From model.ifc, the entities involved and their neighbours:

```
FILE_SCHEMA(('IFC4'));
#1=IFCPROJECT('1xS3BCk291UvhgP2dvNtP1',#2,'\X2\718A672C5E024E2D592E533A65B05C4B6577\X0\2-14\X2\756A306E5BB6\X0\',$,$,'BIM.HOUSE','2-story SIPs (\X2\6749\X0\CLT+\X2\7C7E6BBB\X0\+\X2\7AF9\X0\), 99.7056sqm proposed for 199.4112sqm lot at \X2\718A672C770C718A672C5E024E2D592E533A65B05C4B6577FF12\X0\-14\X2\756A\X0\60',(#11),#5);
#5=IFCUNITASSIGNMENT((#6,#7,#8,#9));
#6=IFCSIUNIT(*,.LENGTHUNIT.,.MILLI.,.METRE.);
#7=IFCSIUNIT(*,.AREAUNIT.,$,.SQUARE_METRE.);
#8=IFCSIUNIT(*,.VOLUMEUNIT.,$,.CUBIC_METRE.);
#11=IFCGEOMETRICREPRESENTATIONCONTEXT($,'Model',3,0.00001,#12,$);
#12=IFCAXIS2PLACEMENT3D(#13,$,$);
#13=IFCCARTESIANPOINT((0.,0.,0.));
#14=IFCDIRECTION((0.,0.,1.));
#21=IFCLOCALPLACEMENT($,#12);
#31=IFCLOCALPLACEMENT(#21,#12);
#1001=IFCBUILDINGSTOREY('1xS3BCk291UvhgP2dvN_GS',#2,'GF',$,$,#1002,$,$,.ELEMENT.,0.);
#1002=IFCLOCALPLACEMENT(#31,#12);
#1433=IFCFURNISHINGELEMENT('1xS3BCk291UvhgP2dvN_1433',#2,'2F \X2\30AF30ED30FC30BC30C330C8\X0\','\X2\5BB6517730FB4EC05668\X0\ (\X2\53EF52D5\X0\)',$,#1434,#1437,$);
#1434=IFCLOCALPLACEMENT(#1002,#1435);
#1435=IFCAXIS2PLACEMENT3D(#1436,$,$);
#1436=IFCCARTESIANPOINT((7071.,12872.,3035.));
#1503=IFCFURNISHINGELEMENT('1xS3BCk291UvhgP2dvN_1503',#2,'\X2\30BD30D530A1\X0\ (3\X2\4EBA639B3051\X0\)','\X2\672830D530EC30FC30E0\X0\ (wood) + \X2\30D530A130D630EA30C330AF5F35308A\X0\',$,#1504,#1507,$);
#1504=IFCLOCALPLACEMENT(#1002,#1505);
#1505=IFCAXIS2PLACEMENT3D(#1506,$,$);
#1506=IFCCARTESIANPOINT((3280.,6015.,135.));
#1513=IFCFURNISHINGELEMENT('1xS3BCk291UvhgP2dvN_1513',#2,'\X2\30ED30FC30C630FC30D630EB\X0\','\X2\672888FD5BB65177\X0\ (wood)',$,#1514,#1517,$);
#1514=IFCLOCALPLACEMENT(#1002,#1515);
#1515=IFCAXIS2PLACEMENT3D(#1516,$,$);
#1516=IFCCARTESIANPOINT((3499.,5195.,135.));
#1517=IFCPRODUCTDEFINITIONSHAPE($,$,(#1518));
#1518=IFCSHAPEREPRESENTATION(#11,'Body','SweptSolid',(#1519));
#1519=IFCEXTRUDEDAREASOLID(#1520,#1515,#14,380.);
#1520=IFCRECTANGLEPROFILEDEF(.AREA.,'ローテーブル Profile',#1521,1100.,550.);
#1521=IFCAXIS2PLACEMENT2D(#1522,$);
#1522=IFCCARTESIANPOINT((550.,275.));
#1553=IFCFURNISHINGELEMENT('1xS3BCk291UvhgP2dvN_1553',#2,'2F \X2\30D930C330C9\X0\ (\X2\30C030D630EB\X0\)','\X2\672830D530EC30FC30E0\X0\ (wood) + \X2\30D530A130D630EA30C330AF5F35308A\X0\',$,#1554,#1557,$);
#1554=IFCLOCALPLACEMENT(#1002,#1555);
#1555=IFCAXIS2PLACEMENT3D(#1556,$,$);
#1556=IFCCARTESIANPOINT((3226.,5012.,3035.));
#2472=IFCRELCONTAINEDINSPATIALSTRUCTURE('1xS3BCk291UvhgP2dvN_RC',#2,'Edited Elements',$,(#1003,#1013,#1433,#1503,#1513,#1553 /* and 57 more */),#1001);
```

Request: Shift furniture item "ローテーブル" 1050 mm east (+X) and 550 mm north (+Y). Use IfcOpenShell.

```python
import ifcopenshell
import ifcopenshell.api.geometry
import ifcopenshell.util.placement
import ifcopenshell.util.unit

model = ifcopenshell.open("model.ifc")
unit_scale = ifcopenshell.util.unit.calculate_unit_scale(model)

item = model.by_guid("1xS3BCk291UvhgP2dvN_1513")
matrix = ifcopenshell.util.placement.get_local_placement(item.ObjectPlacement)
matrix[0, 3] += 1.05 / unit_scale
matrix[1, 3] += 0.55 / unit_scale
ifcopenshell.api.geometry.edit_object_placement(model, product=item, matrix=matrix, is_si=False)

print(ifcopenshell.util.placement.get_local_placement(item.ObjectPlacement).round(3) + 0.0)

model.write("model_v2.ifc")
```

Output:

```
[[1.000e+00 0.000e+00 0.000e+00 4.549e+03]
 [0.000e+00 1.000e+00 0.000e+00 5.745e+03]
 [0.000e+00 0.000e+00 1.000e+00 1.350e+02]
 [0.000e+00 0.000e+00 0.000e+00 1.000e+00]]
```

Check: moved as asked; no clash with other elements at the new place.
